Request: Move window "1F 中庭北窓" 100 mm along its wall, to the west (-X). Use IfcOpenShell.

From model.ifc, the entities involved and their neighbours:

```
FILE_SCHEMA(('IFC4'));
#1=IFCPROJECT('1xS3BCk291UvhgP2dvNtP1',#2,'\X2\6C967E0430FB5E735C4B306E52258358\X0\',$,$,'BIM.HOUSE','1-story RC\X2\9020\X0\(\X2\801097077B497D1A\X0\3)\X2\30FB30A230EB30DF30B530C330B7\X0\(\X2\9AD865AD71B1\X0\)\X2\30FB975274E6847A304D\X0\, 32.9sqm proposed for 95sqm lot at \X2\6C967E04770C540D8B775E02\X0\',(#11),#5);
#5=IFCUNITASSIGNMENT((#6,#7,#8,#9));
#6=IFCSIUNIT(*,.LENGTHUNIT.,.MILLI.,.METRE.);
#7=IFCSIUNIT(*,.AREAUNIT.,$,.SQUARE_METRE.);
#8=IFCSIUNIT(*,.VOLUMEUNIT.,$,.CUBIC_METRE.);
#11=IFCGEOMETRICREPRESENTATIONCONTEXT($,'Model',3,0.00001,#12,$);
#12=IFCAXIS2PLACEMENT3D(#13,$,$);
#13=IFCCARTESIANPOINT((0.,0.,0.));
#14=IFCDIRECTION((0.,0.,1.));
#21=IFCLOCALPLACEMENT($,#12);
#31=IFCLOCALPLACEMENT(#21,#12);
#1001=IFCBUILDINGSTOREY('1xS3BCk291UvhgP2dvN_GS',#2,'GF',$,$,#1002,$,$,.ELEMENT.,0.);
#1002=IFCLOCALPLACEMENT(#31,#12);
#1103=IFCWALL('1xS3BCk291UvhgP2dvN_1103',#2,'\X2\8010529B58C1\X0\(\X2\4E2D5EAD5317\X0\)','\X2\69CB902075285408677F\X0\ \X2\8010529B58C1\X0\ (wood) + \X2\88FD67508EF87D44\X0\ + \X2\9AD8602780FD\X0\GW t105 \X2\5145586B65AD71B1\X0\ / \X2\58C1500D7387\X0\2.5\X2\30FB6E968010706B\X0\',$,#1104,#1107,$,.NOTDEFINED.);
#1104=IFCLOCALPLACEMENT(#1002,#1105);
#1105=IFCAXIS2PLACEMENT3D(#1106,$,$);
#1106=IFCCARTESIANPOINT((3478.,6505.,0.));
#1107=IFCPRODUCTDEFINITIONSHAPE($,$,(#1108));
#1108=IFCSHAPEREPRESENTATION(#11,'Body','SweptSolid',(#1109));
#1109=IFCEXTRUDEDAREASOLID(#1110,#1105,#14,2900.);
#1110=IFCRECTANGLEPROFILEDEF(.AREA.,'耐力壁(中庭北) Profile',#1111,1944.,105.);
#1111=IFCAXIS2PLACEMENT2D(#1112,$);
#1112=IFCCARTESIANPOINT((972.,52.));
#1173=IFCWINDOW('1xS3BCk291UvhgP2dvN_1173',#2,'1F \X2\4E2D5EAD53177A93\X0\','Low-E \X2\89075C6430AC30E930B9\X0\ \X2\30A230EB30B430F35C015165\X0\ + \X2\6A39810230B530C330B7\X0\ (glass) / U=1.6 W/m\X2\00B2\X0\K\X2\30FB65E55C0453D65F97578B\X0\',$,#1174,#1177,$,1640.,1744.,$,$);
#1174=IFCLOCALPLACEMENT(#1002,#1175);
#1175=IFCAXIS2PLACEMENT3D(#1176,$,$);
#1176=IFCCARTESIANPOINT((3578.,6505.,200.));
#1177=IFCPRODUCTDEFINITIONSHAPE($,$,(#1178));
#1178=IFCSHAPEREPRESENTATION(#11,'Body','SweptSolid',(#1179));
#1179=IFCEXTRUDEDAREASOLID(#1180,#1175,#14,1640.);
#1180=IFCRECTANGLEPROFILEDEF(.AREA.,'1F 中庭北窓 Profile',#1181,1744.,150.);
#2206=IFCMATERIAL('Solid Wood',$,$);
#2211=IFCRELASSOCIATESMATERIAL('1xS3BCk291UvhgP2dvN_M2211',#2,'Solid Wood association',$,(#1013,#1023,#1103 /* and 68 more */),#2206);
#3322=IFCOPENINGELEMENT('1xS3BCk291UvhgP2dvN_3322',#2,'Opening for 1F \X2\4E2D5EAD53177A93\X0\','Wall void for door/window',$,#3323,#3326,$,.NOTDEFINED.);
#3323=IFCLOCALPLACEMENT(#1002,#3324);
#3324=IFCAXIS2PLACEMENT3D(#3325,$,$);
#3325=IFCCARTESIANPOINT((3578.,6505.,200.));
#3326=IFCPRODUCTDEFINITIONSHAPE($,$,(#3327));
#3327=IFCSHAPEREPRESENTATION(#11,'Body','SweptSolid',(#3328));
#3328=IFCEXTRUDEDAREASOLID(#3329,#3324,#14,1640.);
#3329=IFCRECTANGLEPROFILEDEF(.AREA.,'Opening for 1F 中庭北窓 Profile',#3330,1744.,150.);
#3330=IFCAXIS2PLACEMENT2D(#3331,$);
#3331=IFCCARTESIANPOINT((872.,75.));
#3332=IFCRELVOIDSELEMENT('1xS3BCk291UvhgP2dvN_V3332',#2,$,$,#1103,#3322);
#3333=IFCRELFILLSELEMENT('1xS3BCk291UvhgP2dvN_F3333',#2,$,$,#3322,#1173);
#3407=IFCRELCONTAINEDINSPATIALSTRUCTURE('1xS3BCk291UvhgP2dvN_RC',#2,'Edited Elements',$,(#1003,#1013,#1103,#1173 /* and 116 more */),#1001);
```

```python
import ifcopenshell
import ifcopenshell.api.geometry
import ifcopenshell.util.placement

model = ifcopenshell.open("model.ifc")

window = model.by_guid("1xS3BCk291UvhgP2dvN_1173")
opening = window.FillsVoids[0].RelatingOpeningElement
wall = opening.VoidsElements[0].RelatingBuildingElement

wall_matrix = ifcopenshell.util.placement.get_local_placement(wall.ObjectPlacement)
shift = wall_matrix[:3, 0] * -100.0
before = ifcopenshell.util.placement.get_local_placement(window.ObjectPlacement)[:3, 3].copy()

# The window is not placed relative to its opening, so move both.
for product in (opening, window):
    matrix = ifcopenshell.util.placement.get_local_placement(product.ObjectPlacement)
    matrix[:3, 3] += shift
    ifcopenshell.api.geometry.edit_object_placement(model, product=product, matrix=matrix, is_si=False)

after = ifcopenshell.util.placement.get_local_placement(window.ObjectPlacement)[:3, 3]
print("window moved by", (after - before).round(3) + 0.0)

model.write("model_edited.ifc")
```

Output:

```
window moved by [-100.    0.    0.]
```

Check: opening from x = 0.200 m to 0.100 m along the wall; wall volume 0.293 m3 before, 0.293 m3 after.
